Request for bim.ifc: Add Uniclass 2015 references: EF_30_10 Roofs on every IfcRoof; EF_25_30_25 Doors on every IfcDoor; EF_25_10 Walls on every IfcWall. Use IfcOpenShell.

First a look at what the model holds.

```python
import ifcopenshell

model = ifcopenshell.open("bim.ifc")
print(model.schema)
print("classifications:", [c.Name for c in model.by_type("IfcClassification")])
for ifc_class in ("IfcDoor", "IfcRoof", "IfcStair", "IfcWall", "IfcWindow"):
    print(ifc_class, len(model.by_type(ifc_class)))
```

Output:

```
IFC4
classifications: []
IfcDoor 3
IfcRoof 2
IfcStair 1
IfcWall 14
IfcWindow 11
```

```python
import ifcopenshell
import ifcopenshell.api.classification

model = ifcopenshell.open("bim.ifc")

system = ifcopenshell.api.classification.add_classification(model, classification="Uniclass 2015")

codes = {
    "IfcRoof": ("EF_30_10", "Roofs"),
    "IfcDoor": ("EF_25_30_25", "Doors"),
    "IfcWall": ("EF_25_10", "Walls"),
}
for ifc_class, (code, name) in codes.items():
    products = model.by_type(ifc_class)
    ifcopenshell.api.classification.add_reference(
        model, products=products, classification=system, identification=code, name=name
    )
    print(code, len(products))

model.write("bim_rev.ifc")
```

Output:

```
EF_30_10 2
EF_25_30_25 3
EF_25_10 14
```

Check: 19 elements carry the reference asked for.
